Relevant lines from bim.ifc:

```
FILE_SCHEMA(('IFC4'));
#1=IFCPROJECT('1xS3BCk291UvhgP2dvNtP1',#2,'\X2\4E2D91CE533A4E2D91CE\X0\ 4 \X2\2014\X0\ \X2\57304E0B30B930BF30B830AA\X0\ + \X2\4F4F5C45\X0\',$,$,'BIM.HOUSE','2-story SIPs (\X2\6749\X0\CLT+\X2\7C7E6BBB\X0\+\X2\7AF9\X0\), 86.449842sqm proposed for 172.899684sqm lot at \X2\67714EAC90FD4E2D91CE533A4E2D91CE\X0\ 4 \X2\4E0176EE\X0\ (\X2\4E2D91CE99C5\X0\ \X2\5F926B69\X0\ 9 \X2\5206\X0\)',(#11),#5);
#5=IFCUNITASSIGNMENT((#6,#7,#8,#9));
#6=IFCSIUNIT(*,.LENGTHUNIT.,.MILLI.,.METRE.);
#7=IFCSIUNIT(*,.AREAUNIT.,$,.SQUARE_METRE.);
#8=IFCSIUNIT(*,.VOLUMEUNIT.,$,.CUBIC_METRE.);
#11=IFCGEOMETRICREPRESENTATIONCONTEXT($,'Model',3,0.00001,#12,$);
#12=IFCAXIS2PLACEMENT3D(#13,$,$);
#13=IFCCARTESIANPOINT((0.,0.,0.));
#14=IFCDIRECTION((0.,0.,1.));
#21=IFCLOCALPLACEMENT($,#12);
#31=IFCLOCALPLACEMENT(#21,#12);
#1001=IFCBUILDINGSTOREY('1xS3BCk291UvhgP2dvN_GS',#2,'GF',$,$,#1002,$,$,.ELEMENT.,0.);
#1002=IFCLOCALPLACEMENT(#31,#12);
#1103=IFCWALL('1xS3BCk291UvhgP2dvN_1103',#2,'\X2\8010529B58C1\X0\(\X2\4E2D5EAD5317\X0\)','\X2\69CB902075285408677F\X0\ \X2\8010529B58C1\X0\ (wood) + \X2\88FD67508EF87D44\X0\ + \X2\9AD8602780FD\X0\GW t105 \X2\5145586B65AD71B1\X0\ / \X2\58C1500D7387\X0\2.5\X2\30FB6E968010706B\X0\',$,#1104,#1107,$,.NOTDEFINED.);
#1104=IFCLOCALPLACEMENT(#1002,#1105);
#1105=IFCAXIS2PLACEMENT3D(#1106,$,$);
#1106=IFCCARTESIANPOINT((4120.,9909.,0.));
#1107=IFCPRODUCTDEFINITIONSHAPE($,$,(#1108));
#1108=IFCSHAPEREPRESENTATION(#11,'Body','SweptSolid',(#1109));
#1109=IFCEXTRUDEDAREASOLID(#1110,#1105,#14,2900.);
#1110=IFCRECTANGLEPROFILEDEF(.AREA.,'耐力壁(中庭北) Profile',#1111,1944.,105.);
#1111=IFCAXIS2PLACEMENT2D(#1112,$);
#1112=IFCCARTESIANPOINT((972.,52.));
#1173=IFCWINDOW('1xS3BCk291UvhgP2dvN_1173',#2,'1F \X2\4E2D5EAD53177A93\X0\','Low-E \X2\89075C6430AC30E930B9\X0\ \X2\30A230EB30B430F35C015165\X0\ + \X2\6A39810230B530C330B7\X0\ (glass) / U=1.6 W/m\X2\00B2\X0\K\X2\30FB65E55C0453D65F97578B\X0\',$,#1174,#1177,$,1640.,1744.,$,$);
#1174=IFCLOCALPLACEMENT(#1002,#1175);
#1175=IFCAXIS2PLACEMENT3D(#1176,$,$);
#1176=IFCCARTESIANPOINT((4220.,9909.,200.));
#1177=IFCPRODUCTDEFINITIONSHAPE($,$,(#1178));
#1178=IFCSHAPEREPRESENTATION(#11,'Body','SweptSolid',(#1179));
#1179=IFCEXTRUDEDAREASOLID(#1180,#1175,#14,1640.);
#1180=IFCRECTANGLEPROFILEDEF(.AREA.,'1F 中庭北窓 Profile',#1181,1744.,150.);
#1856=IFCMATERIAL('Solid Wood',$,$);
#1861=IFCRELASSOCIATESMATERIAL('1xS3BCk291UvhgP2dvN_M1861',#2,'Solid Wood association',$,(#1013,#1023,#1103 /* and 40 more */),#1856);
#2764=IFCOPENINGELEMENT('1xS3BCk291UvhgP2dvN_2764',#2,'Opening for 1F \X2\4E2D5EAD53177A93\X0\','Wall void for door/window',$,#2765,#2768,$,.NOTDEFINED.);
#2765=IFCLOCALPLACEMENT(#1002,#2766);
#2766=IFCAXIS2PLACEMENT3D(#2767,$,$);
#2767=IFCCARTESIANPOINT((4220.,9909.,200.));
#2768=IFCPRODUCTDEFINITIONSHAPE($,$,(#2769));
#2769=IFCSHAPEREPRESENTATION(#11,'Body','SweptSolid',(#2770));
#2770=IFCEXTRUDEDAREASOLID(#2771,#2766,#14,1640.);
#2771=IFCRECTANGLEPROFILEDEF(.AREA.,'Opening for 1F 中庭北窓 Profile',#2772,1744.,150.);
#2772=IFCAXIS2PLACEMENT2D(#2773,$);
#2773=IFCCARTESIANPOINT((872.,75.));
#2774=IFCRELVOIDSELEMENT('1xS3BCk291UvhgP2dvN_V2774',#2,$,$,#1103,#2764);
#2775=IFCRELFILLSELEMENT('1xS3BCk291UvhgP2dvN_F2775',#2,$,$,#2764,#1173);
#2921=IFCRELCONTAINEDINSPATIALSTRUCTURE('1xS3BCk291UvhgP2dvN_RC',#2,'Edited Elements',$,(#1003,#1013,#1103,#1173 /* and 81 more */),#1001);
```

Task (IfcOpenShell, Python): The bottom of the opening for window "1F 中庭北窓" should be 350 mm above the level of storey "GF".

```python
import numpy as np
import ifcopenshell
import ifcopenshell.api.geometry
import ifcopenshell.geom
import ifcopenshell.util.element
import ifcopenshell.util.placement
import ifcopenshell.util.shape
import ifcopenshell.util.unit

model = ifcopenshell.open("bim.ifc")
unit_scale = ifcopenshell.util.unit.calculate_unit_scale(model)

window = model.by_guid("1xS3BCk291UvhgP2dvN_1173")
opening = window.FillsVoids[0].RelatingOpeningElement
storey = ifcopenshell.util.element.get_container(window, ifc_class="IfcBuildingStorey")
level = ifcopenshell.util.placement.get_local_placement(storey.ObjectPlacement)[2, 3]

# The opening's origin need not be at the sill, so measure its lowest point.
shape = ifcopenshell.geom.create_shape(ifcopenshell.geom.settings(), opening)
bottom = ifcopenshell.util.shape.get_shape_bottom_elevation(shape, shape.geometry) / unit_scale
dz = level + 0.35 / unit_scale - bottom

shift = np.array([0.0, 0.0, dz])
# The window is not placed relative to its opening, so move both.
for product in (opening, window):
    matrix = ifcopenshell.util.placement.get_local_placement(product.ObjectPlacement)
    matrix[:3, 3] += shift
    ifcopenshell.api.geometry.edit_object_placement(model, product=product, matrix=matrix, is_si=False)

print(f"moved by {dz * unit_scale:+.3f} m")

model.write("bim_rev.ifc")
```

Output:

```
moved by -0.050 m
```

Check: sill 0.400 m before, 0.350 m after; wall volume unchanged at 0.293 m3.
